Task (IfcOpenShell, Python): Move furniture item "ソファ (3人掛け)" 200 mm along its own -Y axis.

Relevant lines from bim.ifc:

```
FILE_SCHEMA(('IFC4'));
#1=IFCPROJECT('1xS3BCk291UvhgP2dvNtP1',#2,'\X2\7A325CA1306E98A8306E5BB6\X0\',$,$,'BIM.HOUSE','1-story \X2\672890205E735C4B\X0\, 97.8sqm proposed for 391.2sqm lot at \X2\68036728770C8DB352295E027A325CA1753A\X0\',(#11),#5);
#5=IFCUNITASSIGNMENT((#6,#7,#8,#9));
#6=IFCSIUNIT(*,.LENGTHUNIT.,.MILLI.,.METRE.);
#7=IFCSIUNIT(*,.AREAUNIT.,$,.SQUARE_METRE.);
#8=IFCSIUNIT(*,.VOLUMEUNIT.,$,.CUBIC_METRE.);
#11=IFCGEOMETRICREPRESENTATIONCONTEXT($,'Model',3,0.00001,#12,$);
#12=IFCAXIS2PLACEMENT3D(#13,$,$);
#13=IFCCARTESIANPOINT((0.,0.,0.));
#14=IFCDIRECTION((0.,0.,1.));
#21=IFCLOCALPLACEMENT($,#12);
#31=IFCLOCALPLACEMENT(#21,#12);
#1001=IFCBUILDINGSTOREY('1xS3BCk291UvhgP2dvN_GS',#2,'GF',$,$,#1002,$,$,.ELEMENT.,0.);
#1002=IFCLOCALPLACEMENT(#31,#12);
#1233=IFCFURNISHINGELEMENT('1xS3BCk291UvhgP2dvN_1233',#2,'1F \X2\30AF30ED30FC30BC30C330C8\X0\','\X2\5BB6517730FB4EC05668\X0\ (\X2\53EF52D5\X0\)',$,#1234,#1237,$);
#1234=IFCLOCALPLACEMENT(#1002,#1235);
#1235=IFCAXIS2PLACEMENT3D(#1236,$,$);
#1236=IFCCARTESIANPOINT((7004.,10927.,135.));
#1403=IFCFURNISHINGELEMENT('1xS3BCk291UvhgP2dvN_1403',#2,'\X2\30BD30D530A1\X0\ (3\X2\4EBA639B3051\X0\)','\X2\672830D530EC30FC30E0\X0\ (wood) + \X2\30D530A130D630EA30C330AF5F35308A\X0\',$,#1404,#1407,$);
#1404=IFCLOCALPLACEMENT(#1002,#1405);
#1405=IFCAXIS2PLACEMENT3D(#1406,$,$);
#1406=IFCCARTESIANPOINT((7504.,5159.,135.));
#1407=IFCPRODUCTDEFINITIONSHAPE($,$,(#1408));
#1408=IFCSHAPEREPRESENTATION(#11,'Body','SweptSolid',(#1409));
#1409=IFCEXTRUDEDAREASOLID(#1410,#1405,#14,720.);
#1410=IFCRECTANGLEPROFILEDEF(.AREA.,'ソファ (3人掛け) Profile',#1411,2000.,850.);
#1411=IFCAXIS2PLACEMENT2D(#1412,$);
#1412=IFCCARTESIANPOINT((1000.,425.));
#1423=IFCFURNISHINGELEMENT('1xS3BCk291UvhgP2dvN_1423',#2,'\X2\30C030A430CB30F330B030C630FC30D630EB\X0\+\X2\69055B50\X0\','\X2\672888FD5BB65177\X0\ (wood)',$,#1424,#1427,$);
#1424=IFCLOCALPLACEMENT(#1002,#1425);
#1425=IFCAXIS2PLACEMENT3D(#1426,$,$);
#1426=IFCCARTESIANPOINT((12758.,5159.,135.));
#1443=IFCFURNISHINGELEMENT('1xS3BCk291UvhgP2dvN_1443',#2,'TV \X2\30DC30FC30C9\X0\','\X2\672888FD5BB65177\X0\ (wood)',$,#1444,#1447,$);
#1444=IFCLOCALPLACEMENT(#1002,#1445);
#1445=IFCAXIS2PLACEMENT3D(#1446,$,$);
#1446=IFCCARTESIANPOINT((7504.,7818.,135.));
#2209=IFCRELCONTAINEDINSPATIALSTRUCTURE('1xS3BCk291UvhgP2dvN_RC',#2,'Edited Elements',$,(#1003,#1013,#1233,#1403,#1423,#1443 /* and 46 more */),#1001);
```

```python
import ifcopenshell
import ifcopenshell.api.geometry
import ifcopenshell.util.placement
import ifcopenshell.util.unit

model = ifcopenshell.open("bim.ifc")
unit_scale = ifcopenshell.util.unit.calculate_unit_scale(model)

item = model.by_id(1403)
matrix = ifcopenshell.util.placement.get_local_placement(item.ObjectPlacement)
matrix[:3, 3] -= matrix[:3, 1] * 0.2 / unit_scale
ifcopenshell.api.geometry.edit_object_placement(model, product=item, matrix=matrix, is_si=False)

print(ifcopenshell.util.placement.get_local_placement(item.ObjectPlacement).round(3) + 0.0)

model.write("bim_updated.ifc")
```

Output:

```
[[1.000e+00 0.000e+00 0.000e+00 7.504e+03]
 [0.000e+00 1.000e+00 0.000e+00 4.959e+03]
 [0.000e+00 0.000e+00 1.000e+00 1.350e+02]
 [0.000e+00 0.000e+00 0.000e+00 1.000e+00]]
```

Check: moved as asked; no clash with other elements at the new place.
